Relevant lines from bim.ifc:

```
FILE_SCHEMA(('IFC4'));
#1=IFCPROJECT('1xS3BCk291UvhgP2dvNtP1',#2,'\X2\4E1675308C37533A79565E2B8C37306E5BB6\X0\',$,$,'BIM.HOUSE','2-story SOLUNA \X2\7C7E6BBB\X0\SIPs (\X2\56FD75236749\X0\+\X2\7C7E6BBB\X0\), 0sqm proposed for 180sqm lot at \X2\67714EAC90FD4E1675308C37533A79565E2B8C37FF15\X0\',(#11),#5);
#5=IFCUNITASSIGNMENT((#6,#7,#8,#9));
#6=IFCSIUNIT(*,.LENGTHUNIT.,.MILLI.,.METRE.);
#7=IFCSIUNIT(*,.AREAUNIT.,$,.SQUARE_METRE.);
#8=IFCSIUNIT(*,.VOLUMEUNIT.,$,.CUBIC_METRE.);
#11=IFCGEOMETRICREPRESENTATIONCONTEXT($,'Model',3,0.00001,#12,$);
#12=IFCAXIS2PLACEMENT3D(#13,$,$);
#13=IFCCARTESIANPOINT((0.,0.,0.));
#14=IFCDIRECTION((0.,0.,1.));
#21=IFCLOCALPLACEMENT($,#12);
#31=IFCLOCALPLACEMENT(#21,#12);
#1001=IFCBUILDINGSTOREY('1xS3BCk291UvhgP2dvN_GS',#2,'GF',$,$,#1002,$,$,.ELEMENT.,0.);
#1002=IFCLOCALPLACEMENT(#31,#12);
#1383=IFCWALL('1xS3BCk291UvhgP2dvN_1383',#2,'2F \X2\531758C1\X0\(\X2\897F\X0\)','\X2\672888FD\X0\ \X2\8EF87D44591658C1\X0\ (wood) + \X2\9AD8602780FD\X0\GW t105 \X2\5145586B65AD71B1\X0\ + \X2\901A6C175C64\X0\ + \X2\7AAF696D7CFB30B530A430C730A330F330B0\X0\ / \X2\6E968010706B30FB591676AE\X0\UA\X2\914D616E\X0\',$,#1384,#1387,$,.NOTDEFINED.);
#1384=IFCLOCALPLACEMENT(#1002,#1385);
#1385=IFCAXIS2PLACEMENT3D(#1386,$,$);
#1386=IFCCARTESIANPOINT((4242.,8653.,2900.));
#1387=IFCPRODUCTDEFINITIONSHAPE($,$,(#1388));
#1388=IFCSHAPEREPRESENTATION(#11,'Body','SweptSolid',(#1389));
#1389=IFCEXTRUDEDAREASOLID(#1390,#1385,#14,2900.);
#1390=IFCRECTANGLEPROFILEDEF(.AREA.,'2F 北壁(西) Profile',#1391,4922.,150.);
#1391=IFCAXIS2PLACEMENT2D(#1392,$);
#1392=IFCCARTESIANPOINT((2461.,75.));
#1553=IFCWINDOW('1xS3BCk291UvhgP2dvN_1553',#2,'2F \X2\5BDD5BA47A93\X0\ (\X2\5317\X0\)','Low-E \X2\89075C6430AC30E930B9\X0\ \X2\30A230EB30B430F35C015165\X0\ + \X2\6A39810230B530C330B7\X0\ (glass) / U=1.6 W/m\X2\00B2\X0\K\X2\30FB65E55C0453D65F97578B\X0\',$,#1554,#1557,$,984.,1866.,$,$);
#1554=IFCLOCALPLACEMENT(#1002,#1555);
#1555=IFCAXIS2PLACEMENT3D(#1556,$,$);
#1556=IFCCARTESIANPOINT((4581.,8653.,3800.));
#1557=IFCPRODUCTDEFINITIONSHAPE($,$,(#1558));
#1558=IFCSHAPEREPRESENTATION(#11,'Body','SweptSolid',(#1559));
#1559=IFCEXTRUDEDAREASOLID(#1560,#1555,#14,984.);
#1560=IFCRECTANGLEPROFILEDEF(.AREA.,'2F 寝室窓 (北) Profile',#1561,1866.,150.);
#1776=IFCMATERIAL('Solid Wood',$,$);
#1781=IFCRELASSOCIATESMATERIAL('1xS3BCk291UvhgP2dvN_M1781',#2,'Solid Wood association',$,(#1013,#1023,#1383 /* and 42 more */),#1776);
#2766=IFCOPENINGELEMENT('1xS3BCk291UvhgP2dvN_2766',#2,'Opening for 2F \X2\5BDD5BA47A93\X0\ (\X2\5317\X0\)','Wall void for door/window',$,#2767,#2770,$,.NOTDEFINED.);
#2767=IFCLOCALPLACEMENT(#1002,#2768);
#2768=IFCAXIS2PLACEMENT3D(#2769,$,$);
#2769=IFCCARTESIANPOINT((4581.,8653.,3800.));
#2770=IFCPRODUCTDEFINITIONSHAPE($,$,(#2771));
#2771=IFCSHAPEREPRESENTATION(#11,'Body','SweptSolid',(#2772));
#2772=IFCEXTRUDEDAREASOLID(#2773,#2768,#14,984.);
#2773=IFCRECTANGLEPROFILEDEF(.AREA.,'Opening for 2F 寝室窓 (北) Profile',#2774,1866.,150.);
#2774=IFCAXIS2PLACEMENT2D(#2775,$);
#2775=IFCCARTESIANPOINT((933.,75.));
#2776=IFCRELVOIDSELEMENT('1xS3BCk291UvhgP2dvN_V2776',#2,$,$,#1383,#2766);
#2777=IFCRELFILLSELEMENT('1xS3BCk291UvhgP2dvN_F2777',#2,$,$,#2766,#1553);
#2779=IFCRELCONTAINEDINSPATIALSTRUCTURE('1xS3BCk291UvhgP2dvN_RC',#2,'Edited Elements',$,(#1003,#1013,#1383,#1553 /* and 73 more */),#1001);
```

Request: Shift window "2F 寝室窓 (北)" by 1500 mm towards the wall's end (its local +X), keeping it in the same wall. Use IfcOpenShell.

```python
import ifcopenshell
import ifcopenshell.api.geometry
import ifcopenshell.util.placement
import ifcopenshell.util.unit

model = ifcopenshell.open("bim.ifc")
unit_scale = ifcopenshell.util.unit.calculate_unit_scale(model)

window = model.by_guid("1xS3BCk291UvhgP2dvN_1553")
opening = window.FillsVoids[0].RelatingOpeningElement
wall = opening.VoidsElements[0].RelatingBuildingElement

wall_matrix = ifcopenshell.util.placement.get_local_placement(wall.ObjectPlacement)
shift = wall_matrix[:3, 0] * 1.5 / unit_scale
before = ifcopenshell.util.placement.get_local_placement(window.ObjectPlacement)[:3, 3].copy()

# The window is not placed relative to its opening, so move both.
for product in (opening, window):
    matrix = ifcopenshell.util.placement.get_local_placement(product.ObjectPlacement)
    matrix[:3, 3] += shift
    ifcopenshell.api.geometry.edit_object_placement(model, product=product, matrix=matrix, is_si=False)

after = ifcopenshell.util.placement.get_local_placement(window.ObjectPlacement)[:3, 3]
print("window moved by", (after - before).round(3) + 0.0)

model.write("bim_updated.ifc")
```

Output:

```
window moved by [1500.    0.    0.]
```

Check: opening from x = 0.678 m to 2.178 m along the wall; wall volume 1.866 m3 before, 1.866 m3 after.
